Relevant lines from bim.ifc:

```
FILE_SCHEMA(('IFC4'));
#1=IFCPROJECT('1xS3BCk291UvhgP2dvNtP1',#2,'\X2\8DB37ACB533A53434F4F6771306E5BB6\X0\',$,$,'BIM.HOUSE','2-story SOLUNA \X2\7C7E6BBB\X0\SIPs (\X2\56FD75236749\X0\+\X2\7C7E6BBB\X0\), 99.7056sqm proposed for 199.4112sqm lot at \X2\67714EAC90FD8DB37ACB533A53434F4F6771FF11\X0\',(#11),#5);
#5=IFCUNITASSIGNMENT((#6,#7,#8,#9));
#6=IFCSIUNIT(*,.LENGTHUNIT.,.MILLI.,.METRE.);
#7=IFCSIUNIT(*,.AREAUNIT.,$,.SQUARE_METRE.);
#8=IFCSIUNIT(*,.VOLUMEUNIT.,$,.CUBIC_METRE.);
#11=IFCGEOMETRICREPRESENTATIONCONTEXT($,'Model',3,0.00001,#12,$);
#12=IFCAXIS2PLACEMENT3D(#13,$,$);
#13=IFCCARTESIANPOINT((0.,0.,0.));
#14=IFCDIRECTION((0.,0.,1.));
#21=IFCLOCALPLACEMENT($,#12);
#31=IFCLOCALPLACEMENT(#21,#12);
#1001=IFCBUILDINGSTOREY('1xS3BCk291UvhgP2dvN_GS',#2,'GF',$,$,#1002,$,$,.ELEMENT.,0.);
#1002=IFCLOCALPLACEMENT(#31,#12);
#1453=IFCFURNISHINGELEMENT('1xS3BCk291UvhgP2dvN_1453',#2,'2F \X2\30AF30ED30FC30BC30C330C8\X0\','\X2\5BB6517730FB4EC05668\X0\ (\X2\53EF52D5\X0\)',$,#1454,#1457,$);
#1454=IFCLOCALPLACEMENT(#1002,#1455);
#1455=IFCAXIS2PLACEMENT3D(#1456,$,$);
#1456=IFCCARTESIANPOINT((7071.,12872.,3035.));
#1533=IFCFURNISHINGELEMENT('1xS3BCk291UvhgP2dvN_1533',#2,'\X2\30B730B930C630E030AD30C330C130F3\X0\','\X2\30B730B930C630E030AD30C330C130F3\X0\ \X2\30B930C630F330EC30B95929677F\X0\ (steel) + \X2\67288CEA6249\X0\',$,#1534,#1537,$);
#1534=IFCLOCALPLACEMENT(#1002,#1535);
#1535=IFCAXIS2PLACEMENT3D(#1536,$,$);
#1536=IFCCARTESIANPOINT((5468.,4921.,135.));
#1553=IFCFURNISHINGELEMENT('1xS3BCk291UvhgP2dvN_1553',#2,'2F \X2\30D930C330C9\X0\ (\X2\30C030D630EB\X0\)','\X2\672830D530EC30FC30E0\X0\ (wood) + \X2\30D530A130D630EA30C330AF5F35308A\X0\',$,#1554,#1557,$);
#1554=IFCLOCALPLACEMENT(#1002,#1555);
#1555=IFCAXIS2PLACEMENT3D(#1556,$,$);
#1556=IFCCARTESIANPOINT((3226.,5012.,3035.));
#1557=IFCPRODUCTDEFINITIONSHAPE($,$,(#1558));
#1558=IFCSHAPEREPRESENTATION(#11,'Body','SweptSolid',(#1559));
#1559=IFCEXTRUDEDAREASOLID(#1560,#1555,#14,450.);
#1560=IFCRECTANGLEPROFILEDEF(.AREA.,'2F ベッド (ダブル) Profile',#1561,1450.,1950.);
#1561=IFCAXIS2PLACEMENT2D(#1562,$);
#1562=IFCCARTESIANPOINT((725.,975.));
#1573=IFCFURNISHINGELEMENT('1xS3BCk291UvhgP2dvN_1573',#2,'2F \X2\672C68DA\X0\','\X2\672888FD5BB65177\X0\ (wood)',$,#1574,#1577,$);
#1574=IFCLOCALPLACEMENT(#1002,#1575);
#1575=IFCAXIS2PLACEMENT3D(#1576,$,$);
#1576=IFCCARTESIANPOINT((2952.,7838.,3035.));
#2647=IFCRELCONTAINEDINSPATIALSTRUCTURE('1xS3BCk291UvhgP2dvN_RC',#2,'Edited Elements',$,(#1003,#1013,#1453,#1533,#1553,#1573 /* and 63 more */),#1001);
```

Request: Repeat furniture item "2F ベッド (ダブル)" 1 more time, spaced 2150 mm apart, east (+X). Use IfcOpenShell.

```python
import numpy as np
import ifcopenshell
import ifcopenshell.api.geometry
import ifcopenshell.api.root
import ifcopenshell.util.element
import ifcopenshell.util.placement
import ifcopenshell.util.unit

model = ifcopenshell.open("bim.ifc")
unit_scale = ifcopenshell.util.unit.calculate_unit_scale(model)


def reuse_history(source, copy):
    """copy_class also copies each property set's owner history, people and application; keep the originals."""
    for rel in copy.IsDefinedBy:
        if rel.is_a("IfcRelDefinesByProperties") and (history := rel.RelatingPropertyDefinition.OwnerHistory):
            rel.RelatingPropertyDefinition.OwnerHistory = source.OwnerHistory
            ifcopenshell.util.element.remove_deep2(model, history)


source = model.by_guid("1xS3BCk291UvhgP2dvN_1553")
base = ifcopenshell.util.placement.get_local_placement(source.ObjectPlacement)
step = np.array([1.0, 0.0, 0.0]) * 2.15 / unit_scale

for i in range(1, 2):
    copy = ifcopenshell.api.root.copy_class(model, product=source)
    copy.Representation = ifcopenshell.util.element.copy_deep(
        model, source.Representation, exclude=["IfcGeometricRepresentationContext", "IfcRepresentationMap"]
    )
    reuse_history(source, copy)
    matrix = base.copy()
    matrix[:3, 3] += i * step
    print("added at", matrix[:3, 3].round(3) + 0.0)
    ifcopenshell.api.geometry.edit_object_placement(model, product=copy, matrix=matrix, is_si=False)

model.write("bim_rev.ifc")
```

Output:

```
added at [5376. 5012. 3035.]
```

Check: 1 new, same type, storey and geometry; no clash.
